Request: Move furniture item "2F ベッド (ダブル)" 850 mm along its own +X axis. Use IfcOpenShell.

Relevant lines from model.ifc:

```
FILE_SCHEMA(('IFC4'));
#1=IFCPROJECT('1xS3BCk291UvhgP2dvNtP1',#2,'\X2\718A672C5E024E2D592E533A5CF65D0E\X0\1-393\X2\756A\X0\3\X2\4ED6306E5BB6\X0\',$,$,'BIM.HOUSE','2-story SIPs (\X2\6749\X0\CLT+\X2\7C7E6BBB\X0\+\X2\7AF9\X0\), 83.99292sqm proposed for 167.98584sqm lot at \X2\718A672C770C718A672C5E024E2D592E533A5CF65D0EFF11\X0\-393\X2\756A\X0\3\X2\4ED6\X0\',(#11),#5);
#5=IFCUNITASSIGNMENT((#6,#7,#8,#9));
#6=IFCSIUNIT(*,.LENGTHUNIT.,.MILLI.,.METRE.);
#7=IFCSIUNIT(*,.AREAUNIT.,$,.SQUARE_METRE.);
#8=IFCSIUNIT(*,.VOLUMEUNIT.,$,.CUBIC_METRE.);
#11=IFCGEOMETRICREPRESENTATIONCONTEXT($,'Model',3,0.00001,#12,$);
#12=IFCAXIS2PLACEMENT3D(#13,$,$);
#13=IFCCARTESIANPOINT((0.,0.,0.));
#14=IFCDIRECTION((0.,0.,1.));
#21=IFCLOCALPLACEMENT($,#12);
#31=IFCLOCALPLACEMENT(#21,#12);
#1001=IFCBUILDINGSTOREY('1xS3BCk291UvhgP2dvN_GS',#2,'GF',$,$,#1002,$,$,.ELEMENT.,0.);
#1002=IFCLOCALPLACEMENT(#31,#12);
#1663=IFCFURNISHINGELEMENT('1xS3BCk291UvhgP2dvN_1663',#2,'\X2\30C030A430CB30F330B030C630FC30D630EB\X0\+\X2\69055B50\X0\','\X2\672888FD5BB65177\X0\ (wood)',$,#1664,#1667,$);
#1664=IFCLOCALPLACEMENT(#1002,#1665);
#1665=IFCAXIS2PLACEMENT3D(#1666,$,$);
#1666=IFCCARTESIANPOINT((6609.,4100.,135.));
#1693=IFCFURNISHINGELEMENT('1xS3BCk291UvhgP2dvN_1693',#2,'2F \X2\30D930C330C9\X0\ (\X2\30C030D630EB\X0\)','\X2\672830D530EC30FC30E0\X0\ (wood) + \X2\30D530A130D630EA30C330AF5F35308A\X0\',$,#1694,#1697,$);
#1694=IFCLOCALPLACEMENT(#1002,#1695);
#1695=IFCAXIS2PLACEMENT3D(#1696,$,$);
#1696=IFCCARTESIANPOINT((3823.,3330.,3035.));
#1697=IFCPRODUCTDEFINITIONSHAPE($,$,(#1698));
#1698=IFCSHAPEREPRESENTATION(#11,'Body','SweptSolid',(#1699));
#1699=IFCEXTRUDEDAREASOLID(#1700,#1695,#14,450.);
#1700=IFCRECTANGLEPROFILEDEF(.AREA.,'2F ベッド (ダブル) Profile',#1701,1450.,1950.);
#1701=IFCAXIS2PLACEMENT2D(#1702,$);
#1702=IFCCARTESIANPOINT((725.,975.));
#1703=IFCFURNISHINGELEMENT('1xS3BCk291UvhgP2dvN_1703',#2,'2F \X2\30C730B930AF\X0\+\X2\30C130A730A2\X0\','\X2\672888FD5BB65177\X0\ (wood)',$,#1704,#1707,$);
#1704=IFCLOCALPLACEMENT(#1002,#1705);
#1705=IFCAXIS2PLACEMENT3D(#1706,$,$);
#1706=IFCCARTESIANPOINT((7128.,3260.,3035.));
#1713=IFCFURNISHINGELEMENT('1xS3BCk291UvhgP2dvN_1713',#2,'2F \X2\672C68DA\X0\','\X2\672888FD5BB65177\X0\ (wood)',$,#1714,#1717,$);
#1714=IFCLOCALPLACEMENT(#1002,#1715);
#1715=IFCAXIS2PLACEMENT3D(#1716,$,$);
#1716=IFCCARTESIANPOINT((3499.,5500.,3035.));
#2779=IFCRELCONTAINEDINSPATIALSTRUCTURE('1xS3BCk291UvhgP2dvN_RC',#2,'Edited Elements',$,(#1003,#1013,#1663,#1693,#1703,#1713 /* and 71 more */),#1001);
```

```python
import ifcopenshell
import ifcopenshell.api.geometry
import ifcopenshell.util.placement

model = ifcopenshell.open("model.ifc")

item = model.by_id(1693)
matrix = ifcopenshell.util.placement.get_local_placement(item.ObjectPlacement)
matrix[:3, 3] += matrix[:3, 0] * 850.0
ifcopenshell.api.geometry.edit_object_placement(model, product=item, matrix=matrix, is_si=False)

print(ifcopenshell.util.placement.get_local_placement(item.ObjectPlacement).round(3) + 0.0)

model.write("model-out.ifc")
```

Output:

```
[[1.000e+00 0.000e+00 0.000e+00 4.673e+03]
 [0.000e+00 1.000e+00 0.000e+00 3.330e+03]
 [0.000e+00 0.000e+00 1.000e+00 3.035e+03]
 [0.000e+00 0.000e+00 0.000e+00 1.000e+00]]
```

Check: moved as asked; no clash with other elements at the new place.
